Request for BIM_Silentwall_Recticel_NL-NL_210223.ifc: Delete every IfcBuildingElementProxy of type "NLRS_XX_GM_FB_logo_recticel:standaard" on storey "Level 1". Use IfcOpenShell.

First a look at what the model holds.

```python
import ifcopenshell
import ifcopenshell.util.element

model = ifcopenshell.open("BIM_Silentwall_Recticel_NL-NL_210223.ifc")
print(model.schema)
storey = next(s for s in model.by_type("IfcBuildingStorey") if s.Name == "Level 1")
proxies = [e for e in ifcopenshell.util.element.get_decomposition(storey) if e.is_a("IfcBuildingElementProxy")]
seen = {}
for e in proxies:
    element_type = ifcopenshell.util.element.get_type(e)
    name = element_type.Name if element_type not in (None, e) else None
    seen[name] = seen.get(name, 0) + 1
for name, count in sorted(seen.items(), key=str):
    print(count, "x", name)
```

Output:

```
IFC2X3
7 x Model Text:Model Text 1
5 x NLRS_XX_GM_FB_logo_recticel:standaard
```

```python
import ifcopenshell
import ifcopenshell.api.root
import ifcopenshell.util.element

model = ifcopenshell.open("BIM_Silentwall_Recticel_NL-NL_210223.ifc")

storey = next(s for s in model.by_type("IfcBuildingStorey") if s.Name == "Level 1")
proxies = [e for e in ifcopenshell.util.element.get_decomposition(storey) if e.is_a("IfcBuildingElementProxy")]
targets = [e for e in proxies if (t := ifcopenshell.util.element.get_type(e)) not in (None, e) and t.Name == "NLRS_XX_GM_FB_logo_recticel:standaard"]

for e in targets:
    ifcopenshell.api.root.remove_product(model, product=e)
print(len(targets), "removed")

model.write("BIM_Silentwall_Recticel_NL-NL_210223_updated.ifc")
```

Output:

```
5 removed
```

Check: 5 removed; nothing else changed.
